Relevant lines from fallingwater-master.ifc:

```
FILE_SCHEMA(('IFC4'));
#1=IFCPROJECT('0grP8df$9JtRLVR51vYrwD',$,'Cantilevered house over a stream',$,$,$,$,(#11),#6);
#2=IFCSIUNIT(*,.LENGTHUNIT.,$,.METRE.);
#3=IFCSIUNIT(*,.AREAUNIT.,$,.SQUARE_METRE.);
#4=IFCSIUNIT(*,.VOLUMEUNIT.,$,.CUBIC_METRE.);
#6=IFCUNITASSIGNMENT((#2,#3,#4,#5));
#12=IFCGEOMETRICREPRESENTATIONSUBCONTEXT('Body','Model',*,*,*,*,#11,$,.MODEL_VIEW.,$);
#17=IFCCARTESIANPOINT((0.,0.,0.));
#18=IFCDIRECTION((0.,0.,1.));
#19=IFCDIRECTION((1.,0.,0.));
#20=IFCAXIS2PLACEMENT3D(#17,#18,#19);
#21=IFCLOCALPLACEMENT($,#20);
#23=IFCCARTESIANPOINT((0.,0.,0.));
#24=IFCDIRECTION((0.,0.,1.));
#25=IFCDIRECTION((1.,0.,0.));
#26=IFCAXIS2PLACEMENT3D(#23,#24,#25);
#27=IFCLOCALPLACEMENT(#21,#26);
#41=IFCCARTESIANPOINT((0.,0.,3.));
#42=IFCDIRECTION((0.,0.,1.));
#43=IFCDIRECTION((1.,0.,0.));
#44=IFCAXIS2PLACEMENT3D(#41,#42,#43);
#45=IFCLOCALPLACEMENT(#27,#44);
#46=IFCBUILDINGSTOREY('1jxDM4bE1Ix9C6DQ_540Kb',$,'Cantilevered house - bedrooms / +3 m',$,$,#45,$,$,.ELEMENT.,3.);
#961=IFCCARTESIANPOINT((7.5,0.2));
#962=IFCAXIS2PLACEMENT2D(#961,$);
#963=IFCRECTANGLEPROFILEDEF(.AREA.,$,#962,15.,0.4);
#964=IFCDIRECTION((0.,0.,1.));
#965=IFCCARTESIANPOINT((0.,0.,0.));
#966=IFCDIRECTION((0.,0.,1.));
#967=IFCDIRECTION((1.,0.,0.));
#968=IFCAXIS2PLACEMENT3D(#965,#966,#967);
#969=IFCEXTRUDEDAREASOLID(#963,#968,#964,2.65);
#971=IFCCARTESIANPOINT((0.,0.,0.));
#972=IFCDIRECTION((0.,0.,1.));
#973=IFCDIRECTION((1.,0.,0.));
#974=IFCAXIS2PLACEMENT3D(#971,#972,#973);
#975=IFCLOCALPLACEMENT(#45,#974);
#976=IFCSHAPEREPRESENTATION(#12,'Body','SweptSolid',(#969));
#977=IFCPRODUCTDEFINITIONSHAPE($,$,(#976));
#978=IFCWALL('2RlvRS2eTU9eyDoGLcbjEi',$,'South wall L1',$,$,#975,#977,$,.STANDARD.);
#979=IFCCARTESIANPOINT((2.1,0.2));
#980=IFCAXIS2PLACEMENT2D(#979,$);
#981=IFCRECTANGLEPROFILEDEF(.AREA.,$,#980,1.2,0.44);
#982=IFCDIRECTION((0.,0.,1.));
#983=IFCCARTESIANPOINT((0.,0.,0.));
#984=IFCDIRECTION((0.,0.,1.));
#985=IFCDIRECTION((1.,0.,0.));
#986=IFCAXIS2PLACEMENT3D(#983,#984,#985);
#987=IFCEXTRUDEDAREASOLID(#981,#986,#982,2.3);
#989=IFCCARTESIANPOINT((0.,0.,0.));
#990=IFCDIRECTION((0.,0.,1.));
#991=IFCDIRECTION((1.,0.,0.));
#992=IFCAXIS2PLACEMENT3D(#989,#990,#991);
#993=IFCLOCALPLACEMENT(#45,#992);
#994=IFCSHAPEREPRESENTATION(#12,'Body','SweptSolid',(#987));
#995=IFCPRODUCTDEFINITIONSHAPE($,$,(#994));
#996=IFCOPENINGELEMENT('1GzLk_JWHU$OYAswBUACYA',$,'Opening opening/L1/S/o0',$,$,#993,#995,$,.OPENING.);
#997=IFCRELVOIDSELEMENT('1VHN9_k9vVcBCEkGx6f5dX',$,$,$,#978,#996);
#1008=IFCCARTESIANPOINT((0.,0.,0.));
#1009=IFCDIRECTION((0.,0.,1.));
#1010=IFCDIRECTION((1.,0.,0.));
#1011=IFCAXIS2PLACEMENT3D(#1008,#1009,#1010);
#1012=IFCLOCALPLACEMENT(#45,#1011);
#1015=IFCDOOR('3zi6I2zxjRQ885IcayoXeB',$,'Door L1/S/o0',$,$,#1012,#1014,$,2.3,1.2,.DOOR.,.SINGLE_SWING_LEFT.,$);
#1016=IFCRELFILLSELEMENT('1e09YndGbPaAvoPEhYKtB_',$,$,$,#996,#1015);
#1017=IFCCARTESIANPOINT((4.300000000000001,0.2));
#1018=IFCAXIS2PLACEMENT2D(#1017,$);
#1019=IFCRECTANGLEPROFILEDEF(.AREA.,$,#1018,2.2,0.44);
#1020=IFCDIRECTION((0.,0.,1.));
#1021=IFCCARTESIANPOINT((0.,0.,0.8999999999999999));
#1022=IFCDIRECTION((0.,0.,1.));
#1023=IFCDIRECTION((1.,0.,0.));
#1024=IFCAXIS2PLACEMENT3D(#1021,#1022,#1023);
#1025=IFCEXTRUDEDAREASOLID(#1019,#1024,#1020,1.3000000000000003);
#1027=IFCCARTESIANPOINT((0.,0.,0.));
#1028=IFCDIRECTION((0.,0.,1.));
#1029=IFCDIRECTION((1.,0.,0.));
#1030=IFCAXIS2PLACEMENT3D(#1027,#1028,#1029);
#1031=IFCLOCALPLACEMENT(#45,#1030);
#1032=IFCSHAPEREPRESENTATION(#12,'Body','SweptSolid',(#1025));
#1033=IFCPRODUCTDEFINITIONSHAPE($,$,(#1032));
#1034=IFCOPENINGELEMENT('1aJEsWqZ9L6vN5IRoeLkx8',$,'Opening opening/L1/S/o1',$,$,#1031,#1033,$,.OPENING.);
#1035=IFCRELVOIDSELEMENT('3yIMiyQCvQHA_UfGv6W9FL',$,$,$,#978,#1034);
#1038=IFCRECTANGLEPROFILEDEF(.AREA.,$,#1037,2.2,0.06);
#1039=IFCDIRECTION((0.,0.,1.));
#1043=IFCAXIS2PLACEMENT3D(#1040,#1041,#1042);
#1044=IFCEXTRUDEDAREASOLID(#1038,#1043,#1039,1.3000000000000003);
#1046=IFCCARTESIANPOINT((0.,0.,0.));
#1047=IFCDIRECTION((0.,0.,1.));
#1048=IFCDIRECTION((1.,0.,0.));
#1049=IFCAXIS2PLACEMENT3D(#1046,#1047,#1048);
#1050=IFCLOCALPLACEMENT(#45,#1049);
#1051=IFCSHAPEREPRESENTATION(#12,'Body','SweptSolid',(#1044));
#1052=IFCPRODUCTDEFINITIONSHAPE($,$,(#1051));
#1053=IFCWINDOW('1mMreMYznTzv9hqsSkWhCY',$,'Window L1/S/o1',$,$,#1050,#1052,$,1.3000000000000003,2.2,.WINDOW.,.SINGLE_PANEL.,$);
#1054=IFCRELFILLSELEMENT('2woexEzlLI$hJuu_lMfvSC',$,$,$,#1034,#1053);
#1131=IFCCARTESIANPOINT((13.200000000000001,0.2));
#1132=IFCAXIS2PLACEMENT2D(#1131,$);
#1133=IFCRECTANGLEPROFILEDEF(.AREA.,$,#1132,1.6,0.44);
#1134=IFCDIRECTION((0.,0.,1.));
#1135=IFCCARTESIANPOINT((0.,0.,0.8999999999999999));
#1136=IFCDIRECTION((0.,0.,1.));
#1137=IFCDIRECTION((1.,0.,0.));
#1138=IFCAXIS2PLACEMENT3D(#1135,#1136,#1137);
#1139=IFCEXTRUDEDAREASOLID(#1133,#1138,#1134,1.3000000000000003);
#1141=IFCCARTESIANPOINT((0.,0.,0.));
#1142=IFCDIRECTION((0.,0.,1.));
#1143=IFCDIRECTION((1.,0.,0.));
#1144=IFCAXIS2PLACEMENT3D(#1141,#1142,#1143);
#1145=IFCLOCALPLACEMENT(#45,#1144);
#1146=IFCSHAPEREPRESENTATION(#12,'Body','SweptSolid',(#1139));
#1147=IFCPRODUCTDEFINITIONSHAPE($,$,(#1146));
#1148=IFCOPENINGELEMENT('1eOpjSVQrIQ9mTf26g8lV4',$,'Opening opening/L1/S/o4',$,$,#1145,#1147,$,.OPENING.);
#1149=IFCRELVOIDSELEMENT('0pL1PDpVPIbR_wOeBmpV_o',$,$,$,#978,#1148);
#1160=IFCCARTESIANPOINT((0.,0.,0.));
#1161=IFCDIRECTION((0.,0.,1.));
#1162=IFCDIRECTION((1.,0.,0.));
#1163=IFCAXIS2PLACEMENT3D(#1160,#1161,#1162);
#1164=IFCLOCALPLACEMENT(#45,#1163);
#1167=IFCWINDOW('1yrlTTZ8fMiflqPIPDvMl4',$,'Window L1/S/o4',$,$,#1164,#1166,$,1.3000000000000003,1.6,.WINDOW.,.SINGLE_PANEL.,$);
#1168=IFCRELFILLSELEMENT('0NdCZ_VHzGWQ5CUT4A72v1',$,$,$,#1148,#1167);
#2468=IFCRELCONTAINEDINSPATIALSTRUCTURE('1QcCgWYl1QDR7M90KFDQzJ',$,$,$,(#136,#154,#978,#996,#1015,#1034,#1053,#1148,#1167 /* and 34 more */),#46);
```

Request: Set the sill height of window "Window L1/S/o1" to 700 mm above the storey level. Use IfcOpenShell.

```python
import numpy as np
import ifcopenshell
import ifcopenshell.api.geometry
import ifcopenshell.geom
import ifcopenshell.util.element
import ifcopenshell.util.placement
import ifcopenshell.util.shape
import ifcopenshell.util.unit

model = ifcopenshell.open("fallingwater-master.ifc")
unit_scale = ifcopenshell.util.unit.calculate_unit_scale(model)

window = model.by_id(1053)
opening = window.FillsVoids[0].RelatingOpeningElement
storey = ifcopenshell.util.element.get_container(window, ifc_class="IfcBuildingStorey")
level = ifcopenshell.util.placement.get_local_placement(storey.ObjectPlacement)[2, 3]

# The opening's origin need not be at the sill, so measure its lowest point.
shape = ifcopenshell.geom.create_shape(ifcopenshell.geom.settings(), opening)
bottom = ifcopenshell.util.shape.get_shape_bottom_elevation(shape, shape.geometry) / unit_scale
dz = level + 0.7 - bottom

shift = np.array([0.0, 0.0, dz])
# The window is not placed relative to its opening, so move both.
for product in (opening, window):
    matrix = ifcopenshell.util.placement.get_local_placement(product.ObjectPlacement)
    matrix[:3, 3] += shift
    ifcopenshell.api.geometry.edit_object_placement(model, product=product, matrix=matrix, is_si=False)

print(f"moved by {dz * unit_scale:+.3f} m")

model.write("fallingwater-master_rev.ifc")
```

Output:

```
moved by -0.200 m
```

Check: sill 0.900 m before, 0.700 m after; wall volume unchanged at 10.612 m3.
